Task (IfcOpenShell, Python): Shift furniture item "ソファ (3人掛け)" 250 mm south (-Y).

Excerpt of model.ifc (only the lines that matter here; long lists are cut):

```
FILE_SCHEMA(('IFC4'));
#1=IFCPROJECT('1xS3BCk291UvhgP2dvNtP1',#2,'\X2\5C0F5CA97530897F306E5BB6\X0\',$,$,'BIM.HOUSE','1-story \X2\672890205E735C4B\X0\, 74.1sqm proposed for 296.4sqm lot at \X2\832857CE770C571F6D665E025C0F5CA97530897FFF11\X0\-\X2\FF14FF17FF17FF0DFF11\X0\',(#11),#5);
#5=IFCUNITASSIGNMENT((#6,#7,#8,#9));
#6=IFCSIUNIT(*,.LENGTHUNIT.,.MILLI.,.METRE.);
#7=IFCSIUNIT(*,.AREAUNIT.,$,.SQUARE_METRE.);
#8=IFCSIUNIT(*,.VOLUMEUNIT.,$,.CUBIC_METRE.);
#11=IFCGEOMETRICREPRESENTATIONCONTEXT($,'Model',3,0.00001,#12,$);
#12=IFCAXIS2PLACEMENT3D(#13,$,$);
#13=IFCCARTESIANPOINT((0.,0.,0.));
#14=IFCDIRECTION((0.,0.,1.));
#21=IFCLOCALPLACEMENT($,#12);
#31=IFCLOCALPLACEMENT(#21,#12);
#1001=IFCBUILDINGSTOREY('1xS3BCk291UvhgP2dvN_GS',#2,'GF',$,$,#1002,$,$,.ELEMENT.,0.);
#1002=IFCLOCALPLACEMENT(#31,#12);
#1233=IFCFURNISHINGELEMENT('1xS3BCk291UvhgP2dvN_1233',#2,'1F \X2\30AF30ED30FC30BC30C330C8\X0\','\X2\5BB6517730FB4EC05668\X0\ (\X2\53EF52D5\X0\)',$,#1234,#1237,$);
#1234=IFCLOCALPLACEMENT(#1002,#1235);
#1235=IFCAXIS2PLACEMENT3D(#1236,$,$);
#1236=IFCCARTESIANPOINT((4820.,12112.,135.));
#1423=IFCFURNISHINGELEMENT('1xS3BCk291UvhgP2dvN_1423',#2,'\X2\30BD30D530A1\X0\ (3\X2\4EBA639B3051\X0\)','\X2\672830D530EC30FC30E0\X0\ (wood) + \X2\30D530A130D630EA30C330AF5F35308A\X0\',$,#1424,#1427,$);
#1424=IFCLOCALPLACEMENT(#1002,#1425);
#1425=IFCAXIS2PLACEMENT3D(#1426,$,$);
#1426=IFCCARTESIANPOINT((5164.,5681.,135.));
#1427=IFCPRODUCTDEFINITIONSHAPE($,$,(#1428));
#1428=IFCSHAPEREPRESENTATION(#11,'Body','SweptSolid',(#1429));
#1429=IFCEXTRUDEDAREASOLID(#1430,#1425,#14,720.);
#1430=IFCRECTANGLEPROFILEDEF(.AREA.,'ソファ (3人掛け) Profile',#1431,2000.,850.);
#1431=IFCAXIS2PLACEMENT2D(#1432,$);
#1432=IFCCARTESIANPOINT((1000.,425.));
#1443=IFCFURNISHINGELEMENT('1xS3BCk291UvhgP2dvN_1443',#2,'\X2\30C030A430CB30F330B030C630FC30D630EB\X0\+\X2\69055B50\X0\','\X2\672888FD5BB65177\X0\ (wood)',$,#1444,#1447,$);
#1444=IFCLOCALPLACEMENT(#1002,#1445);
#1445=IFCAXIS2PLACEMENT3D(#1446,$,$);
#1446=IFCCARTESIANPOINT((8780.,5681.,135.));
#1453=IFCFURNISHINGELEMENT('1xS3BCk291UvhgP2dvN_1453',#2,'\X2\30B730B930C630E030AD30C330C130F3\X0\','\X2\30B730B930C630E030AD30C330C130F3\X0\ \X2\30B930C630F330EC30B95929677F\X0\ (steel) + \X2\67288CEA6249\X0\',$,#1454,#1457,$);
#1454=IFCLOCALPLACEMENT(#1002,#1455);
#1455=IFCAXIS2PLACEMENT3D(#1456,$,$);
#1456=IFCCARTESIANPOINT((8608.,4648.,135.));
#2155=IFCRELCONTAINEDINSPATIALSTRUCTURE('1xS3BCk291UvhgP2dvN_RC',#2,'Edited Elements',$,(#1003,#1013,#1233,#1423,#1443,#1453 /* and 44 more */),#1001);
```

```python
import ifcopenshell
import ifcopenshell.api.geometry
import ifcopenshell.util.placement

model = ifcopenshell.open("model.ifc")

item = model.by_guid("1xS3BCk291UvhgP2dvN_1423")
matrix = ifcopenshell.util.placement.get_local_placement(item.ObjectPlacement)
matrix[1, 3] -= 250.0
ifcopenshell.api.geometry.edit_object_placement(model, product=item, matrix=matrix, is_si=False)

print(ifcopenshell.util.placement.get_local_placement(item.ObjectPlacement).round(3) + 0.0)

model.write("model_updated.ifc")
```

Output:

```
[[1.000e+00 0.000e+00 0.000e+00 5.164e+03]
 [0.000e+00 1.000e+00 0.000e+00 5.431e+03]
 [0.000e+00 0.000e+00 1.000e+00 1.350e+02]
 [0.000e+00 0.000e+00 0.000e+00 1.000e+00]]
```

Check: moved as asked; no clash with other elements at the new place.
